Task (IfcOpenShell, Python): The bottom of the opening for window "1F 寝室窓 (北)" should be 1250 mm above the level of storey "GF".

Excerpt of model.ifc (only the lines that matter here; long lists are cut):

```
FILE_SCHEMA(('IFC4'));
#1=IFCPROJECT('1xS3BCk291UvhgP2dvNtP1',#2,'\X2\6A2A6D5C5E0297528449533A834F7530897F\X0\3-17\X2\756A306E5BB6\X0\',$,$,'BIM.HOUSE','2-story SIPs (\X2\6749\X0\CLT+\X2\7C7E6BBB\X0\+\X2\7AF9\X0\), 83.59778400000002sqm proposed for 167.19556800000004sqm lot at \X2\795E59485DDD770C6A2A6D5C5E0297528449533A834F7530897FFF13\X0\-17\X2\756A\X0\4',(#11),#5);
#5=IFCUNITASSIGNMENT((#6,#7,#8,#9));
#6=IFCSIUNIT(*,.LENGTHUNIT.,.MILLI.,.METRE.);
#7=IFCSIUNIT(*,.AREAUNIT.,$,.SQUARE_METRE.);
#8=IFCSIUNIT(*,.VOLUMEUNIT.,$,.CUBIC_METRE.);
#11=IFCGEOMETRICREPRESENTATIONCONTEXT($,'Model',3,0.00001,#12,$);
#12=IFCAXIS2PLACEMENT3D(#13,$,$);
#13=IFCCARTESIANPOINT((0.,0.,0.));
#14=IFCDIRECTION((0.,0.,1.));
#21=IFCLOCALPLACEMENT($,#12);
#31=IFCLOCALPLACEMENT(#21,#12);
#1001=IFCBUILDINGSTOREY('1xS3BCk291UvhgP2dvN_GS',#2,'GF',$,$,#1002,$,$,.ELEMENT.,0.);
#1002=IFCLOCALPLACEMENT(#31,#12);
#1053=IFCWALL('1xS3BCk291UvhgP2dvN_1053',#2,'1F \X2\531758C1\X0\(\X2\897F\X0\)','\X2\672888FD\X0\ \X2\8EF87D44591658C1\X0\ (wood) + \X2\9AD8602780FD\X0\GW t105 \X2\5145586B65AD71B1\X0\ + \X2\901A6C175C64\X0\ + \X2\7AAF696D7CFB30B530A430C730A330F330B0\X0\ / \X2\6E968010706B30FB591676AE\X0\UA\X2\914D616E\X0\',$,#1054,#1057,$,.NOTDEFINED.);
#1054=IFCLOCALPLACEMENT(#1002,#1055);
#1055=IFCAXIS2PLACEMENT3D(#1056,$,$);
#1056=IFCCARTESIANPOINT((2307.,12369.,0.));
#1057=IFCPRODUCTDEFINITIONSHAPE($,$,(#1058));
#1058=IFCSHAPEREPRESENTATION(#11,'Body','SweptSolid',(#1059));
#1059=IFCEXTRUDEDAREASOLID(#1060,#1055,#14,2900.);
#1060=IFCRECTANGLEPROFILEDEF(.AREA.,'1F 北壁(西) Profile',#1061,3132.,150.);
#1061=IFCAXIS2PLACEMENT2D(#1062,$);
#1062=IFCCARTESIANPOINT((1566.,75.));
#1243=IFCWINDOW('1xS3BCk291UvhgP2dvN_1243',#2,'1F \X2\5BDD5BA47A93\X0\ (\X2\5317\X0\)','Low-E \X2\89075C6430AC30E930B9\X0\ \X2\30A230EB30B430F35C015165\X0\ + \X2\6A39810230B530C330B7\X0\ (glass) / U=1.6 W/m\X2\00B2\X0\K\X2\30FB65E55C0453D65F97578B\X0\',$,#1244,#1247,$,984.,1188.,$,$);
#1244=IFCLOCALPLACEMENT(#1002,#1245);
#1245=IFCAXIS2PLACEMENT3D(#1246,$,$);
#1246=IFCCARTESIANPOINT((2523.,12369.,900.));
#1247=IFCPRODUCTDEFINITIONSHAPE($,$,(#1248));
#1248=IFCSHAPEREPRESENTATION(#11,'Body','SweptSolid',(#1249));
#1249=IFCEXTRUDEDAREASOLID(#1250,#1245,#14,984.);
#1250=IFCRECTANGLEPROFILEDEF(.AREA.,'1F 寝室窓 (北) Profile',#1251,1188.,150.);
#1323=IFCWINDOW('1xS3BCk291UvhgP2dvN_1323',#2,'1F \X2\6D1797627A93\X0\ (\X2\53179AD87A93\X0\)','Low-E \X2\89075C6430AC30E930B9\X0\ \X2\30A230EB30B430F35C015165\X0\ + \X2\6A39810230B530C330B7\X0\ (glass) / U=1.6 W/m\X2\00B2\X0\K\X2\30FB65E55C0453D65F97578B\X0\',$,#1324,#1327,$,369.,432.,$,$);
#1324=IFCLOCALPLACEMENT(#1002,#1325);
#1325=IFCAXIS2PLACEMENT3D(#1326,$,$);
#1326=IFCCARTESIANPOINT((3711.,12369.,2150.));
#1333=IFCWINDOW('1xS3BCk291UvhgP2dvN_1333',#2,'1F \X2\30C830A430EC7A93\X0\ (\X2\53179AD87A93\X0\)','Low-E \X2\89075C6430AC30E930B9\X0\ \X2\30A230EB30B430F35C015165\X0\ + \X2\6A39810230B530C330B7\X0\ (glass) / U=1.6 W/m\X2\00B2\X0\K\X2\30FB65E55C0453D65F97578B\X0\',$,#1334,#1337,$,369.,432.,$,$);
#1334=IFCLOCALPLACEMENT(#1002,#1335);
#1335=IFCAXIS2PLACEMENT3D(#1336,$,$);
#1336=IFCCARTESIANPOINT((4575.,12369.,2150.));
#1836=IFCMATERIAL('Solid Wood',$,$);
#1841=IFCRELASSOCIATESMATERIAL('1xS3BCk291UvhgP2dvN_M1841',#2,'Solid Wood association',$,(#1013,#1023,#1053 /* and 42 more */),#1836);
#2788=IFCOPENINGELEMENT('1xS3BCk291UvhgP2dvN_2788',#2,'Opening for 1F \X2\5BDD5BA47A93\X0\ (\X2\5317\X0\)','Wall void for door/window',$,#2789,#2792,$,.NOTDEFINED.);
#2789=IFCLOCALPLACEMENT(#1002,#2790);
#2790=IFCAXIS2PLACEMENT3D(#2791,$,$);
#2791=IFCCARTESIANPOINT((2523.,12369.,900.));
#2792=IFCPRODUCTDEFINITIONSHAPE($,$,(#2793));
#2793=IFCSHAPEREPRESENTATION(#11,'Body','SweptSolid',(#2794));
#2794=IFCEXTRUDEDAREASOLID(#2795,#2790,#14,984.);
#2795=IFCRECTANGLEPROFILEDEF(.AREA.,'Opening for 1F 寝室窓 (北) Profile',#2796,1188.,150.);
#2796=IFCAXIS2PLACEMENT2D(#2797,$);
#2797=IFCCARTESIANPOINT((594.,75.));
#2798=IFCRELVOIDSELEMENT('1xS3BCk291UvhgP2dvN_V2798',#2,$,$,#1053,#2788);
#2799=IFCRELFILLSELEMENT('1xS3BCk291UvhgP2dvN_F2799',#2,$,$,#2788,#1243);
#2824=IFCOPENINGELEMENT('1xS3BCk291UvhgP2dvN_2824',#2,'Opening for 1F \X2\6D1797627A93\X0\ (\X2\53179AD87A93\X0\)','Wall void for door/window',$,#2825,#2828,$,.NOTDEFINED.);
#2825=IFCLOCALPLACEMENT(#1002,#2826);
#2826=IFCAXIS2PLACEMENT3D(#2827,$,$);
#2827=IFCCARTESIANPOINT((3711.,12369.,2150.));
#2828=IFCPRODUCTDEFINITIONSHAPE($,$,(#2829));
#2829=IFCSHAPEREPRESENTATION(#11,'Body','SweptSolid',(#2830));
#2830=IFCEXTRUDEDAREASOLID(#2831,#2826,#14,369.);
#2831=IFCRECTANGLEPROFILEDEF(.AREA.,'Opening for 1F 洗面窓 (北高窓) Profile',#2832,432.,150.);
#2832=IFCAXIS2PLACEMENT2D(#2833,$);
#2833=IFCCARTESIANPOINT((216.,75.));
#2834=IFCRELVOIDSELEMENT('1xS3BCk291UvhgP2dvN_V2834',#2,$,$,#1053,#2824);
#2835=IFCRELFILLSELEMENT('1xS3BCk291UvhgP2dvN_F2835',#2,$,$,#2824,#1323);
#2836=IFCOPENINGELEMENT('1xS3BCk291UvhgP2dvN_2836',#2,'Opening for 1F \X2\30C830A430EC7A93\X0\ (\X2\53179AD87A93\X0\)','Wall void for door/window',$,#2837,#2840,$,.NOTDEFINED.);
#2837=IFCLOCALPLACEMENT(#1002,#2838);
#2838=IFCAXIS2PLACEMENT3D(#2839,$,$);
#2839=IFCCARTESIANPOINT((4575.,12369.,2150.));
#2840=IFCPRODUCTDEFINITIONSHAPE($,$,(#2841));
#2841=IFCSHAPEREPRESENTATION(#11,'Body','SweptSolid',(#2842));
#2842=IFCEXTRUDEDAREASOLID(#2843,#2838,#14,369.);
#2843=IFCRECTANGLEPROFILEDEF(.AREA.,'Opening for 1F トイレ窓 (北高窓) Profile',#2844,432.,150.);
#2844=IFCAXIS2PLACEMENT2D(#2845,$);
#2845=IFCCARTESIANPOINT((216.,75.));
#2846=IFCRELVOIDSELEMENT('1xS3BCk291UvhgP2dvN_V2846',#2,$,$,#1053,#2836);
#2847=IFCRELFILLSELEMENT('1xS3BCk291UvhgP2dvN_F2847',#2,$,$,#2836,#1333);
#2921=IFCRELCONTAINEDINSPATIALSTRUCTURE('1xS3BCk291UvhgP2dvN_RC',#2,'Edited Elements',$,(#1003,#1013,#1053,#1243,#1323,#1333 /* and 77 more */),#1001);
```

```python
import numpy as np
import ifcopenshell
import ifcopenshell.api.geometry
import ifcopenshell.geom
import ifcopenshell.util.element
import ifcopenshell.util.placement
import ifcopenshell.util.shape
import ifcopenshell.util.unit

model = ifcopenshell.open("model.ifc")
unit_scale = ifcopenshell.util.unit.calculate_unit_scale(model)

window = model.by_guid("1xS3BCk291UvhgP2dvN_1243")
opening = window.FillsVoids[0].RelatingOpeningElement
storey = ifcopenshell.util.element.get_container(window, ifc_class="IfcBuildingStorey")
level = ifcopenshell.util.placement.get_local_placement(storey.ObjectPlacement)[2, 3]

# The opening's origin need not be at the sill, so measure its lowest point.
shape = ifcopenshell.geom.create_shape(ifcopenshell.geom.settings(), opening)
bottom = ifcopenshell.util.shape.get_shape_bottom_elevation(shape, shape.geometry) / unit_scale
dz = level + 1.25 / unit_scale - bottom

shift = np.array([0.0, 0.0, dz])
# The window is not placed relative to its opening, so move both.
for product in (opening, window):
    matrix = ifcopenshell.util.placement.get_local_placement(product.ObjectPlacement)
    matrix[:3, 3] += shift
    ifcopenshell.api.geometry.edit_object_placement(model, product=product, matrix=matrix, is_si=False)

print(f"moved by {dz * unit_scale:+.3f} m")

model.write("model_edited.ifc")
```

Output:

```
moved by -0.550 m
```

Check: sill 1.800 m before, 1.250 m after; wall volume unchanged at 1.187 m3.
